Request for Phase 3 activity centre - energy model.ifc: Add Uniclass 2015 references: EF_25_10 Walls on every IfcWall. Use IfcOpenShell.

First a look at what the model holds.

```python
import ifcopenshell

model = ifcopenshell.open("Phase 3 activity centre - energy model.ifc")
print(model.schema)
print("classifications:", [c.Name for c in model.by_type("IfcClassification")])
for ifc_class in ("IfcDoor", "IfcRoof", "IfcStair", "IfcWall", "IfcWindow"):
    print(ifc_class, len(model.by_type(ifc_class)))
```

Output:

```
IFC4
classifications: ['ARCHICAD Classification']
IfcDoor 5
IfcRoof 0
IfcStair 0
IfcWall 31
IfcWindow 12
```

```python
import ifcopenshell
import ifcopenshell.api.classification

model = ifcopenshell.open("Phase 3 activity centre - energy model.ifc")

system = ifcopenshell.api.classification.add_classification(model, classification="Uniclass 2015")

codes = {
    "IfcWall": ("EF_25_10", "Walls"),
}
for ifc_class, (code, name) in codes.items():
    products = model.by_type(ifc_class)
    ifcopenshell.api.classification.add_reference(
        model, products=products, classification=system, identification=code, name=name
    )
    print(code, len(products))

model.write("Phase 3 activity centre - energy model_edited.ifc")
```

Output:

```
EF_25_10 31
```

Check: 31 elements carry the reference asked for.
